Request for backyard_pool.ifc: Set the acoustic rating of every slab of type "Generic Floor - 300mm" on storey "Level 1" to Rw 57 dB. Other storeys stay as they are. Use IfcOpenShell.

First a look at what the model holds.

```python
import ifcopenshell
import ifcopenshell.util.element

model = ifcopenshell.open("backyard_pool.ifc")
print(model.schema)
storey = next(s for s in model.by_type("IfcBuildingStorey") if s.Name == "Level 1")
slabs = [e for e in ifcopenshell.util.element.get_decomposition(storey) if e.is_a("IfcSlab")]
seen = {}
for e in slabs:
    element_type = ifcopenshell.util.element.get_type(e)
    key = (element_type.Name if element_type != e and element_type else None, ifcopenshell.util.element.get_pset(e, "Pset_SlabCommon", "AcousticRating"))
    seen[key] = seen.get(key, 0) + 1
for (name, value), count in sorted(seen.items(), key=str):
    print(count, "x", name, "|", value)
```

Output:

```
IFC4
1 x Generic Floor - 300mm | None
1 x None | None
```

```python
import ifcopenshell
import ifcopenshell.api.pset
import ifcopenshell.util.element

model = ifcopenshell.open("backyard_pool.ifc")

storey = next(s for s in model.by_type("IfcBuildingStorey") if s.Name == "Level 1")
slabs = [e for e in ifcopenshell.util.element.get_decomposition(storey) if e.is_a("IfcSlab")]

count = 0
for e in slabs:
    element_type = ifcopenshell.util.element.get_type(e)
    if element_type in (None, e) or element_type.Name != "Generic Floor - 300mm":
        continue
    # add_pset returns the element's existing set when there is one.
    pset = ifcopenshell.api.pset.add_pset(model, product=e, name="Pset_SlabCommon")
    ifcopenshell.api.pset.edit_pset(model, pset=pset, properties={"AcousticRating": "Rw 57 dB"})
    count += 1

print(count, "slabs updated")

model.write("backyard_pool_edited.ifc")
```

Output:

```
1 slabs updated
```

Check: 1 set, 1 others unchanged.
